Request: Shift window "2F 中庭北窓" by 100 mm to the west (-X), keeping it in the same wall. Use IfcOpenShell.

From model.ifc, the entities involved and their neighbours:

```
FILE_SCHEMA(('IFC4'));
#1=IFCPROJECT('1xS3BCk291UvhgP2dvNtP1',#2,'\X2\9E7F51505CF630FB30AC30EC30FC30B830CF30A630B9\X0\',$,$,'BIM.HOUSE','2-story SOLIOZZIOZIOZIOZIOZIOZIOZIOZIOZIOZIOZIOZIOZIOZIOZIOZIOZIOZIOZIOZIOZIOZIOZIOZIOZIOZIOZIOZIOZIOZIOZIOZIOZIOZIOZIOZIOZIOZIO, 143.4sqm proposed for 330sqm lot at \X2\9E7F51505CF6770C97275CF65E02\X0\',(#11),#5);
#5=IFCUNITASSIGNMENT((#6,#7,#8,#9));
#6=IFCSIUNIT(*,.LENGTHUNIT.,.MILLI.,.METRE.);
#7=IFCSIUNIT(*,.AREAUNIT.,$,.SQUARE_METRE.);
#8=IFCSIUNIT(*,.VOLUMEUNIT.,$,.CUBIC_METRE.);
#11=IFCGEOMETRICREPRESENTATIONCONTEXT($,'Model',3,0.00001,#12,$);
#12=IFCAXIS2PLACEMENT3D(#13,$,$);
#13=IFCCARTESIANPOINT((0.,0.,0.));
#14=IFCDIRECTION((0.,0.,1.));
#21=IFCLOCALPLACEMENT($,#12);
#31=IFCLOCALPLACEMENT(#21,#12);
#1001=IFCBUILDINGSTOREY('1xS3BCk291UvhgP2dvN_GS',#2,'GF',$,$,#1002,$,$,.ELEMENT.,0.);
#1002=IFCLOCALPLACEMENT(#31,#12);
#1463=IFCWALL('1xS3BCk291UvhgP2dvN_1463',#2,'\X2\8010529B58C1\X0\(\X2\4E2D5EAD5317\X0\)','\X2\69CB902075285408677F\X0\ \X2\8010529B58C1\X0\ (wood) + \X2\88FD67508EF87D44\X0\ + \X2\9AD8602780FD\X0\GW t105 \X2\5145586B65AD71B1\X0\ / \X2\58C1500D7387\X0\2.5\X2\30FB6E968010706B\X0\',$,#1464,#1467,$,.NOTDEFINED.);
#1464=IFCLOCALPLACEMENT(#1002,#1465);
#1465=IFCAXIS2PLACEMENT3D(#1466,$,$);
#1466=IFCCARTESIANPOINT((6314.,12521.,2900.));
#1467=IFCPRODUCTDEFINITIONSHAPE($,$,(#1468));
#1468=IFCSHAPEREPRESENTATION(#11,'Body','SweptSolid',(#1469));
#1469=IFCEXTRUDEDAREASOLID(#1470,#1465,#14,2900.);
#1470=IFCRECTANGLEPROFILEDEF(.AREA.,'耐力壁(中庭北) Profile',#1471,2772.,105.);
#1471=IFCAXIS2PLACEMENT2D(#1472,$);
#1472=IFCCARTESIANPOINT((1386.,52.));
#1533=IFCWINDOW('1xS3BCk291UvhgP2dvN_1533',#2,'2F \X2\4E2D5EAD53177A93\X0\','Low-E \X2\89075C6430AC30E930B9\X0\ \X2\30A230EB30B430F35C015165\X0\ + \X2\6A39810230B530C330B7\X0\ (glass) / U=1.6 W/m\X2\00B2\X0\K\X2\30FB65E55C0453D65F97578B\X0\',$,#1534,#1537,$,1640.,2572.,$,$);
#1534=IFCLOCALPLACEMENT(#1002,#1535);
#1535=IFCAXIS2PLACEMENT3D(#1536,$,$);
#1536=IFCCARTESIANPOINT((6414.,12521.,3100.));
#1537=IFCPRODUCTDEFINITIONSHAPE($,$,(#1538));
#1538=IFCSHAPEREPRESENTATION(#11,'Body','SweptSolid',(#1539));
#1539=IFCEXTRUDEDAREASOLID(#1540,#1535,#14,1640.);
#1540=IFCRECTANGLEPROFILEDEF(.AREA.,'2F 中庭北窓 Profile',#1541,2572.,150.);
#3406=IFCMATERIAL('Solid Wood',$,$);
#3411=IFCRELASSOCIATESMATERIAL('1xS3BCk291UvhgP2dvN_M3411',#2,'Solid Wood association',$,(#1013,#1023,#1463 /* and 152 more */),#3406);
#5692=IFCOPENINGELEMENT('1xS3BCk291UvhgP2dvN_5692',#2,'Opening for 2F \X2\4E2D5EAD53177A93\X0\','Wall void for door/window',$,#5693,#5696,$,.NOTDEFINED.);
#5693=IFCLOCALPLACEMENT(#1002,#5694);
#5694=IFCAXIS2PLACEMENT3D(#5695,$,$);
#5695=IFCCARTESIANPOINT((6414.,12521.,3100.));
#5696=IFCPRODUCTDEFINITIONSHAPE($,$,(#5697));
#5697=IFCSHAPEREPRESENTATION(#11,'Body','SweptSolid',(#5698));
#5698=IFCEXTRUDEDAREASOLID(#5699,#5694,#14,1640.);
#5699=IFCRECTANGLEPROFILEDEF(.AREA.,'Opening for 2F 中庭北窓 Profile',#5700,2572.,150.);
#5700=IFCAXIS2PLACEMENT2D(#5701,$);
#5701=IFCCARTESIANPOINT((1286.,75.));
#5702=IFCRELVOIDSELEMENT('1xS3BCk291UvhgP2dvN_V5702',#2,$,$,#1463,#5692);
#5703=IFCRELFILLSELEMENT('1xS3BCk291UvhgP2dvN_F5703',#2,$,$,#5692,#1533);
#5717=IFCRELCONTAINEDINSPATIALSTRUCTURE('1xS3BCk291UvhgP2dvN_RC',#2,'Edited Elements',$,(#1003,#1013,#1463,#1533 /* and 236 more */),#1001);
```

```python
import ifcopenshell
import ifcopenshell.api.geometry
import ifcopenshell.util.placement

model = ifcopenshell.open("model.ifc")

window = model.by_guid("1xS3BCk291UvhgP2dvN_1533")
opening = window.FillsVoids[0].RelatingOpeningElement
wall = opening.VoidsElements[0].RelatingBuildingElement

wall_matrix = ifcopenshell.util.placement.get_local_placement(wall.ObjectPlacement)
shift = wall_matrix[:3, 0] * -100.0
before = ifcopenshell.util.placement.get_local_placement(window.ObjectPlacement)[:3, 3].copy()

# The window is not placed relative to its opening, so move both.
for product in (opening, window):
    matrix = ifcopenshell.util.placement.get_local_placement(product.ObjectPlacement)
    matrix[:3, 3] += shift
    ifcopenshell.api.geometry.edit_object_placement(model, product=product, matrix=matrix, is_si=False)

after = ifcopenshell.util.placement.get_local_placement(window.ObjectPlacement)[:3, 3]
print("window moved by", (after - before).round(3) + 0.0)

model.write("model-out.ifc")
```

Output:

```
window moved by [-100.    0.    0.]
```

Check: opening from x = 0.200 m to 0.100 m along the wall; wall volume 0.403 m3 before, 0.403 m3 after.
